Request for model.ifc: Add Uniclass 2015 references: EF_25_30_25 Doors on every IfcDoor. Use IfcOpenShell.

First a look at what the model holds.

```python
import ifcopenshell

model = ifcopenshell.open("model.ifc")
print(model.schema)
print("classifications:", [c.Name for c in model.by_type("IfcClassification")])
for ifc_class in ("IfcDoor", "IfcRoof", "IfcStair", "IfcWall", "IfcWindow"):
    print(ifc_class, len(model.by_type(ifc_class)))
```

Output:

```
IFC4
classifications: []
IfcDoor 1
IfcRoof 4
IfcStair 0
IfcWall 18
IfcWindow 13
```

```python
import ifcopenshell
import ifcopenshell.api.classification

model = ifcopenshell.open("model.ifc")

system = ifcopenshell.api.classification.add_classification(model, classification="Uniclass 2015")

codes = {
    "IfcDoor": ("EF_25_30_25", "Doors"),
}
for ifc_class, (code, name) in codes.items():
    products = model.by_type(ifc_class)
    ifcopenshell.api.classification.add_reference(
        model, products=products, classification=system, identification=code, name=name
    )
    print(code, len(products))

model.write("model_v2.ifc")
```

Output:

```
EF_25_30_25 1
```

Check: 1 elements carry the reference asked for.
